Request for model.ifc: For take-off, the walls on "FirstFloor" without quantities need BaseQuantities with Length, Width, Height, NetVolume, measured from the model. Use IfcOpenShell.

First a look at what the model holds.

```python
import ifcopenshell
import ifcopenshell.util.element
import ifcopenshell.util.unit

model = ifcopenshell.open("model.ifc")
print(model.schema)
for unit_type in ("LENGTHUNIT", "AREAUNIT", "VOLUMEUNIT"):
    print(unit_type, ifcopenshell.util.unit.calculate_unit_scale(model, unit_type))
storey = next(s for s in model.by_type("IfcBuildingStorey") if s.Name == "FirstFloor")
walls = [e for e in ifcopenshell.util.element.get_decomposition(storey) if e.is_a("IfcWall")]
for e in sorted(walls, key=lambda e: e.id()):
    print(e.id(), e.is_a(), e.Name, list(ifcopenshell.util.element.get_psets(e, qtos_only=True)), sep=" | ")
```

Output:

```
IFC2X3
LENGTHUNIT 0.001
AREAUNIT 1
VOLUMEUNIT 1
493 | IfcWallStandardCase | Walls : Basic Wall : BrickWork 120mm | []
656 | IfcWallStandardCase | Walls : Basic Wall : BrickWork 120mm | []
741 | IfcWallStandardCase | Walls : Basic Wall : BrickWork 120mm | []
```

```python
import ifcopenshell
import ifcopenshell.api.pset
import ifcopenshell.geom
import ifcopenshell.util.element
import ifcopenshell.util.shape
import ifcopenshell.util.unit

model = ifcopenshell.open("model.ifc")
unit_scale = ifcopenshell.util.unit.calculate_unit_scale(model)
volume_scale = ifcopenshell.util.unit.calculate_unit_scale(model, "VOLUMEUNIT")
settings = ifcopenshell.geom.settings()

storey = next(s for s in model.by_type("IfcBuildingStorey") if s.Name == "FirstFloor")
walls = [e for e in ifcopenshell.util.element.get_decomposition(storey) if e.is_a("IfcWall")]

for e in sorted(walls, key=lambda e: e.id()):
    if ifcopenshell.util.element.get_psets(e, qtos_only=True, should_inherit=False):
        continue
    # Geometry comes back in metres, in the element's own axes.
    shape = ifcopenshell.geom.create_shape(settings, e)
    values = {
        "Length": ifcopenshell.util.shape.get_x(shape.geometry) / unit_scale,
        "Width": ifcopenshell.util.shape.get_y(shape.geometry) / unit_scale,
        "Height": ifcopenshell.util.shape.get_z(shape.geometry) / unit_scale,
        "NetVolume": ifcopenshell.util.shape.get_volume(shape.geometry) / volume_scale,
    }
    qto = ifcopenshell.api.pset.add_qto(model, product=e, name="BaseQuantities")
    ifcopenshell.api.pset.edit_qto(model, qto=qto, properties=values)
    print(e.id(), {k: round(v, 3) for k, v in values.items()})

model.write("model_updated.ifc")
```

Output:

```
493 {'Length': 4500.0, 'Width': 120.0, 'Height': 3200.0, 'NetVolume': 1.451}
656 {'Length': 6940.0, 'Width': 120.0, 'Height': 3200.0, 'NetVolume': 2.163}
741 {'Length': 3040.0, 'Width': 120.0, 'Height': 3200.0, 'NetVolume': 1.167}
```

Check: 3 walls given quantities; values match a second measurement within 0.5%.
